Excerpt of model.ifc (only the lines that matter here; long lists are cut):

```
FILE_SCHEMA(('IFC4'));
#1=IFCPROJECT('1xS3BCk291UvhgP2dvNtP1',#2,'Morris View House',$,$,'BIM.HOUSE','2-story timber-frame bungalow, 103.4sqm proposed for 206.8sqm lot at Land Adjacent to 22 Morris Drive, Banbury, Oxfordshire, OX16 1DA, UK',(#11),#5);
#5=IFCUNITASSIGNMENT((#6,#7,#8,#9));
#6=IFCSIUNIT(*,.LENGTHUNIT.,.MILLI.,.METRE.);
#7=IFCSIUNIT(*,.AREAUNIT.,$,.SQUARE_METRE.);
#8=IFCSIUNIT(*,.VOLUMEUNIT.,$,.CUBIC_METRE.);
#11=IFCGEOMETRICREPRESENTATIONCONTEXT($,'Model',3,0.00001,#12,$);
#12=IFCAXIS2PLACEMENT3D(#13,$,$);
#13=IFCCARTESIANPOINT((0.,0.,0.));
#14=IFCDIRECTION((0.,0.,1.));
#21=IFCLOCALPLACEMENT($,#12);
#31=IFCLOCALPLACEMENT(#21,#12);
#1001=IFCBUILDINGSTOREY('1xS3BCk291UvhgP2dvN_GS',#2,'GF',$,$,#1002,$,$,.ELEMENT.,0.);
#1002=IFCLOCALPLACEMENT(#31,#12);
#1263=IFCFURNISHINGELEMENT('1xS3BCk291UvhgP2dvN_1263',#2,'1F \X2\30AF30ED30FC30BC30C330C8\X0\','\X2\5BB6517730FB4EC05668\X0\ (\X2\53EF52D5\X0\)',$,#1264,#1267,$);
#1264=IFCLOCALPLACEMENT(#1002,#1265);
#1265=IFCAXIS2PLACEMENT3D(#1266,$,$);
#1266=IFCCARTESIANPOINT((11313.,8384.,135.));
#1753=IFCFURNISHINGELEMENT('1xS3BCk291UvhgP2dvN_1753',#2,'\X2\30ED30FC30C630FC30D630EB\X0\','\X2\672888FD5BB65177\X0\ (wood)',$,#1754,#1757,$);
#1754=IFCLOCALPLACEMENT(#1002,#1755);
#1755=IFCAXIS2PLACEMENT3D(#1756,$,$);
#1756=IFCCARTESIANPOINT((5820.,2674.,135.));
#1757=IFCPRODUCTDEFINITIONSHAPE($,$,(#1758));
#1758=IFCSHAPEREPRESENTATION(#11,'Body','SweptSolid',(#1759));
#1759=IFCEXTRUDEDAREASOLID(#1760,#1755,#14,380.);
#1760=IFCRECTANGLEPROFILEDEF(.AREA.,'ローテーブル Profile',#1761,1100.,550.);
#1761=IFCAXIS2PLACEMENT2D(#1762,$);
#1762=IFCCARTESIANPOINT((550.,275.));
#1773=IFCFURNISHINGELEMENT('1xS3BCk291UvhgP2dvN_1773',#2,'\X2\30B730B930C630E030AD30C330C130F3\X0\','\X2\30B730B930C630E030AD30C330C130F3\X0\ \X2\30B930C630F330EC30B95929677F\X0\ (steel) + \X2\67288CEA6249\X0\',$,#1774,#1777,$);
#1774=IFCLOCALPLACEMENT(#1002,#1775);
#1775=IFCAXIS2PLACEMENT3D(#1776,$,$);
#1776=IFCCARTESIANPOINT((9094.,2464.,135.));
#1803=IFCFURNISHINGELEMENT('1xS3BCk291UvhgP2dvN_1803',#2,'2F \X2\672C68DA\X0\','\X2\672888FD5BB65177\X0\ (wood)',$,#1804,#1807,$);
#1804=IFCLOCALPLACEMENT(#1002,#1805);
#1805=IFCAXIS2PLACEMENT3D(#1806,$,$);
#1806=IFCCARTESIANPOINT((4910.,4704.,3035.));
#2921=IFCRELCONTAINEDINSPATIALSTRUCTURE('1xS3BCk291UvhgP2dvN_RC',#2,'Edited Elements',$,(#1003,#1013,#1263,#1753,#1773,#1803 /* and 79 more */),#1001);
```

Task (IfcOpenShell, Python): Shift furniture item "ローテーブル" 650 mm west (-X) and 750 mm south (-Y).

```python
import ifcopenshell
import ifcopenshell.api.geometry
import ifcopenshell.util.placement

model = ifcopenshell.open("model.ifc")

item = model.by_guid("1xS3BCk291UvhgP2dvN_1753")
matrix = ifcopenshell.util.placement.get_local_placement(item.ObjectPlacement)
matrix[0, 3] -= 650.0
matrix[1, 3] -= 750.0
ifcopenshell.api.geometry.edit_object_placement(model, product=item, matrix=matrix, is_si=False)

print(ifcopenshell.util.placement.get_local_placement(item.ObjectPlacement).round(3) + 0.0)

model.write("model_v2.ifc")
```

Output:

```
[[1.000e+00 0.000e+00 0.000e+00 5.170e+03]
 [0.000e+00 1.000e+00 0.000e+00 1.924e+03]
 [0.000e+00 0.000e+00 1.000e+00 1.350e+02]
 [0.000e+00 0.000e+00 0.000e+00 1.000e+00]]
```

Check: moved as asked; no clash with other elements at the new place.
